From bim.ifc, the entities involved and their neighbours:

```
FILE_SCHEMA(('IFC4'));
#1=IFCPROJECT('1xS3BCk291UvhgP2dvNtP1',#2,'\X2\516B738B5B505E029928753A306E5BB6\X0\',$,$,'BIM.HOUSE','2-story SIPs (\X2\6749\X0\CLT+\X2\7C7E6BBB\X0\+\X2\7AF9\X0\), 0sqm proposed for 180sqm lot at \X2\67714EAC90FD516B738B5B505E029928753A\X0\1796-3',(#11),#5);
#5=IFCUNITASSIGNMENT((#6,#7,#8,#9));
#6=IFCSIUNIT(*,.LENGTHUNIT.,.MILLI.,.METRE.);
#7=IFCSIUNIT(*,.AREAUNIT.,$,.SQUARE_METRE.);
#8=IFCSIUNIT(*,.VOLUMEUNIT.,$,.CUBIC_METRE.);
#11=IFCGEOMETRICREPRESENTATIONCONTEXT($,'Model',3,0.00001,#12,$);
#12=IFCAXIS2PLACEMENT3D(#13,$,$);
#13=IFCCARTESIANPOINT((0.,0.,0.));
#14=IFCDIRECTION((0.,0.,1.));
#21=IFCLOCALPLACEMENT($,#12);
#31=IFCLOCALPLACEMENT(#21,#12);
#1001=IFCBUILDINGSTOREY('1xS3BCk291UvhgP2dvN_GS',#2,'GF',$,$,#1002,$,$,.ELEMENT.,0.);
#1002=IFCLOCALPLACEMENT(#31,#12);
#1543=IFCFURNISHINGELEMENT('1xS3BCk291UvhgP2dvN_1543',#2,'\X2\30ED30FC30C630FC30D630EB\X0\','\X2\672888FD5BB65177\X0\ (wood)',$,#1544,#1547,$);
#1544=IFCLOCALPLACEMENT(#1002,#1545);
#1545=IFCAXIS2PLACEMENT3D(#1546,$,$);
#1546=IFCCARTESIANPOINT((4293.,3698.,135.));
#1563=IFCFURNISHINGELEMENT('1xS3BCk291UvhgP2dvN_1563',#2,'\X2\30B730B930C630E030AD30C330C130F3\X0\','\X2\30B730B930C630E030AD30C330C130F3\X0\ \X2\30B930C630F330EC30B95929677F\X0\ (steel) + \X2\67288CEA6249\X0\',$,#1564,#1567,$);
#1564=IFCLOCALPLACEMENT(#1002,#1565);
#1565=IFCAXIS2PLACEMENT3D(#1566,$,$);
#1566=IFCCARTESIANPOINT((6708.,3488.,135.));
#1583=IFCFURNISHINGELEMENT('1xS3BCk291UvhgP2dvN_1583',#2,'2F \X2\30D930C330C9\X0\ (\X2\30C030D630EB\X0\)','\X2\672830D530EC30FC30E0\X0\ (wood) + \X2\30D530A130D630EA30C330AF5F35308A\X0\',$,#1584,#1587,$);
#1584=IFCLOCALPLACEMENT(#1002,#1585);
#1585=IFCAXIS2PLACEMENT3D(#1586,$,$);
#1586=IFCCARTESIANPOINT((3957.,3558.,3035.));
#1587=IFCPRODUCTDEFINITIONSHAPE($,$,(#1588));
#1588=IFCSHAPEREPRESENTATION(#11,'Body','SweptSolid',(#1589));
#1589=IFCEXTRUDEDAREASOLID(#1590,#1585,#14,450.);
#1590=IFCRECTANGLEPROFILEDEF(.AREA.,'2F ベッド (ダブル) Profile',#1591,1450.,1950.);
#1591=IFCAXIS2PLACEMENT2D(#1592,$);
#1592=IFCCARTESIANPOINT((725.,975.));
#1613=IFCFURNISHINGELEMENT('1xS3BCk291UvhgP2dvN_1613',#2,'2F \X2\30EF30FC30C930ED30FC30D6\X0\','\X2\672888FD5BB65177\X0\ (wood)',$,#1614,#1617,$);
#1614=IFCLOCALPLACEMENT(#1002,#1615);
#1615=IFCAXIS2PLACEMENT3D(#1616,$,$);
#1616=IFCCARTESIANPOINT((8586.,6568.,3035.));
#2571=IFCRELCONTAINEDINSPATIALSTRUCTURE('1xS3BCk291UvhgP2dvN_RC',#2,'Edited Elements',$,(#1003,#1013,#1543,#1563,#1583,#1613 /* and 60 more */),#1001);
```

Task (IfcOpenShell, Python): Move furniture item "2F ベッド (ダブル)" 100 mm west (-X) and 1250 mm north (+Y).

```python
import ifcopenshell
import ifcopenshell.api.geometry
import ifcopenshell.util.placement

model = ifcopenshell.open("bim.ifc")

item = model.by_guid("1xS3BCk291UvhgP2dvN_1583")
matrix = ifcopenshell.util.placement.get_local_placement(item.ObjectPlacement)
matrix[0, 3] -= 100.0
matrix[1, 3] += 1250.0
ifcopenshell.api.geometry.edit_object_placement(model, product=item, matrix=matrix, is_si=False)

print(ifcopenshell.util.placement.get_local_placement(item.ObjectPlacement).round(3) + 0.0)

model.write("bim_v2.ifc")
```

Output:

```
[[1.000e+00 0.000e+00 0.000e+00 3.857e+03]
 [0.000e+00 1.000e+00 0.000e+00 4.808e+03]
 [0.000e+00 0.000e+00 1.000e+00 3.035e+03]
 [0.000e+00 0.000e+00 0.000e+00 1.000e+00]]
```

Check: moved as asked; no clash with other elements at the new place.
